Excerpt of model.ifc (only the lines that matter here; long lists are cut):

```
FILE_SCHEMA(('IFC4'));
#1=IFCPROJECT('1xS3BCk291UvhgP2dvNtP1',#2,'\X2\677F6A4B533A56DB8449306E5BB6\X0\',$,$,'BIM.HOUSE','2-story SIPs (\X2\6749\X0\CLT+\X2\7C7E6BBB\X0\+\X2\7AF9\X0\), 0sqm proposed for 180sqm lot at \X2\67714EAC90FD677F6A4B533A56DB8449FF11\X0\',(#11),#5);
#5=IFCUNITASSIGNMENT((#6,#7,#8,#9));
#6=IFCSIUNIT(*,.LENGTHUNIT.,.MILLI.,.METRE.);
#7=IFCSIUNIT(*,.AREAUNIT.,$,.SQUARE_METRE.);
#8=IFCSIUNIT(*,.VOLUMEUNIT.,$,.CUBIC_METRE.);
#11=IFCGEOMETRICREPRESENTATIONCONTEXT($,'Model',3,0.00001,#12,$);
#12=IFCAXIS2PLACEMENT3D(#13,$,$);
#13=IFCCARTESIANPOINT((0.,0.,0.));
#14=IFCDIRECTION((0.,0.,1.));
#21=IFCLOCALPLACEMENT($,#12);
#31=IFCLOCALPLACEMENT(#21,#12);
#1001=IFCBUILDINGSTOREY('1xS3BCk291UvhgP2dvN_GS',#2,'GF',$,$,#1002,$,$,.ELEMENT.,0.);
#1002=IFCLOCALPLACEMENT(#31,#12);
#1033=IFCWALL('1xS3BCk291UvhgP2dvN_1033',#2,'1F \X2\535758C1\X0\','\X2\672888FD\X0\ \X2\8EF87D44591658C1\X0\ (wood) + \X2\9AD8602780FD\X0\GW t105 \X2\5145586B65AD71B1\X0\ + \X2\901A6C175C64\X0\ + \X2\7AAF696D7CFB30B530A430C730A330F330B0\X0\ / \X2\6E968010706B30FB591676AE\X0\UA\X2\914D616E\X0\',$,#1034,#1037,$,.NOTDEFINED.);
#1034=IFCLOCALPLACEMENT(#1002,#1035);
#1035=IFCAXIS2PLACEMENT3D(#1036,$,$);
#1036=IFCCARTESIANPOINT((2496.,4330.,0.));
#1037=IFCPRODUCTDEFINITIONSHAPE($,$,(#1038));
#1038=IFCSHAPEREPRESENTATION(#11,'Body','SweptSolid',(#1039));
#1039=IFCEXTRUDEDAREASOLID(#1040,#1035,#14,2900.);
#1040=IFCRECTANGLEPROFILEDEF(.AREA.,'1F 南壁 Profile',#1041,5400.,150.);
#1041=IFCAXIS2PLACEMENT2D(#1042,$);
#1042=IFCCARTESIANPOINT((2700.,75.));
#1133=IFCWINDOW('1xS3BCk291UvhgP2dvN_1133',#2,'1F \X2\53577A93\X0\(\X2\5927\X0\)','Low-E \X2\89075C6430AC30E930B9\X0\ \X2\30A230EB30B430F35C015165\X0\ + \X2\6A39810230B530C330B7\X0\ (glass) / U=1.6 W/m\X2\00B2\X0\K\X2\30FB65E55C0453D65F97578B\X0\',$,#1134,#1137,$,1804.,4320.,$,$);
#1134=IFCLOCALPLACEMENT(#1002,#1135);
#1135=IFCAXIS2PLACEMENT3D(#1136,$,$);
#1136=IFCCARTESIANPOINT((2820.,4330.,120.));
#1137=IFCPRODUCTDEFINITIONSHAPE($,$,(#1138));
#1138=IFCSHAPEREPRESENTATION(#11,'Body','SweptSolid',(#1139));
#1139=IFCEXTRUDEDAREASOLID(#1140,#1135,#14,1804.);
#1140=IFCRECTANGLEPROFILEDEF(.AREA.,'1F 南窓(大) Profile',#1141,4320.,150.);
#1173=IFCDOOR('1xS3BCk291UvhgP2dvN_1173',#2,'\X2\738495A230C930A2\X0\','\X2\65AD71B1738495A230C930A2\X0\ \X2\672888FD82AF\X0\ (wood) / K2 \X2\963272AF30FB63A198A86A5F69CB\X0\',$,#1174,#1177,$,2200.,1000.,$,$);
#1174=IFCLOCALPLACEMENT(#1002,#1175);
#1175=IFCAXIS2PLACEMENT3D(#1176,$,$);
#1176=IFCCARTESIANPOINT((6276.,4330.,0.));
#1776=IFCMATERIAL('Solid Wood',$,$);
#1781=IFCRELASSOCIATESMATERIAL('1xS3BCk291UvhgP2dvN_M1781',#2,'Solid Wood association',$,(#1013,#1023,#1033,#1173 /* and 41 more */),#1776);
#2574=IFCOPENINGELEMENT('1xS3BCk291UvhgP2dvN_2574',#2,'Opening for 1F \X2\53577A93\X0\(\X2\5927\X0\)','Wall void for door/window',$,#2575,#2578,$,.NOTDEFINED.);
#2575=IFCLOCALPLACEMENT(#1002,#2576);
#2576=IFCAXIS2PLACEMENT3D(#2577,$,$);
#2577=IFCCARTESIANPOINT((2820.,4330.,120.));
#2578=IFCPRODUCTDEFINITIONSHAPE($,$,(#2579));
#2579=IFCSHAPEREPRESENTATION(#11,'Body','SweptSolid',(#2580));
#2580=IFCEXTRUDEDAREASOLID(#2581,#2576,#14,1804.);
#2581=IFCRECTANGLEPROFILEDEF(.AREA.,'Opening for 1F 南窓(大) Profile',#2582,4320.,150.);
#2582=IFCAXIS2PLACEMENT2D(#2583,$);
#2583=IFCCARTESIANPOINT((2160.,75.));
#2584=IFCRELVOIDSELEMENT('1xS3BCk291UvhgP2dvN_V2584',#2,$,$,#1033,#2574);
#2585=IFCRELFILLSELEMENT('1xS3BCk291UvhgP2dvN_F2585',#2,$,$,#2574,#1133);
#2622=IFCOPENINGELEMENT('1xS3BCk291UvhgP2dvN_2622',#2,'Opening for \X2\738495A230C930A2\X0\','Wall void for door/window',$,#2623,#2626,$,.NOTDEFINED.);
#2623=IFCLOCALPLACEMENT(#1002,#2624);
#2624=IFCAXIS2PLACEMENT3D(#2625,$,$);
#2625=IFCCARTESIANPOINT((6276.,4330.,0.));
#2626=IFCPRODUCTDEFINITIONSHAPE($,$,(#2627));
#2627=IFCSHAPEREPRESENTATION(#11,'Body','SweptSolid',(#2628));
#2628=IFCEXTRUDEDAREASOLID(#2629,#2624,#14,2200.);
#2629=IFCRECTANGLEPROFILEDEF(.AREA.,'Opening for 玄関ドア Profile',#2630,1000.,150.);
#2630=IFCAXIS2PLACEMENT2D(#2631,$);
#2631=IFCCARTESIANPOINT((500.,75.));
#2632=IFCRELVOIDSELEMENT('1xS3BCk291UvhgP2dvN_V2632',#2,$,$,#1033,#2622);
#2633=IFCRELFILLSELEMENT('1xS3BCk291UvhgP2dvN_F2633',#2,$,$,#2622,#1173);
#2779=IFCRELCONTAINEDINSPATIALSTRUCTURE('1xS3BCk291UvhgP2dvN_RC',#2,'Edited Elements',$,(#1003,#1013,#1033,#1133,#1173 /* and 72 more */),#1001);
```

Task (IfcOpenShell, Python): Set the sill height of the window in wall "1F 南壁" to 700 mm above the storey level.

```python
import numpy as np
import ifcopenshell
import ifcopenshell.api.geometry
import ifcopenshell.geom
import ifcopenshell.util.element
import ifcopenshell.util.placement
import ifcopenshell.util.shape
import ifcopenshell.util.unit

model = ifcopenshell.open("model.ifc")
unit_scale = ifcopenshell.util.unit.calculate_unit_scale(model)

window = model.by_guid("1xS3BCk291UvhgP2dvN_1133")
opening = window.FillsVoids[0].RelatingOpeningElement
storey = ifcopenshell.util.element.get_container(window, ifc_class="IfcBuildingStorey")
level = ifcopenshell.util.placement.get_local_placement(storey.ObjectPlacement)[2, 3]

# The opening's origin need not be at the sill, so measure its lowest point.
shape = ifcopenshell.geom.create_shape(ifcopenshell.geom.settings(), opening)
bottom = ifcopenshell.util.shape.get_shape_bottom_elevation(shape, shape.geometry) / unit_scale
dz = level + 0.7 / unit_scale - bottom

shift = np.array([0.0, 0.0, dz])
# The window is not placed relative to its opening, so move both.
for product in (opening, window):
    matrix = ifcopenshell.util.placement.get_local_placement(product.ObjectPlacement)
    matrix[:3, 3] += shift
    ifcopenshell.api.geometry.edit_object_placement(model, product=product, matrix=matrix, is_si=False)

print(f"moved by {dz * unit_scale:+.3f} m")

model.write("model_v2.ifc")
```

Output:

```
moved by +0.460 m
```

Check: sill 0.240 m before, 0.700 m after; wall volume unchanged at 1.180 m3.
